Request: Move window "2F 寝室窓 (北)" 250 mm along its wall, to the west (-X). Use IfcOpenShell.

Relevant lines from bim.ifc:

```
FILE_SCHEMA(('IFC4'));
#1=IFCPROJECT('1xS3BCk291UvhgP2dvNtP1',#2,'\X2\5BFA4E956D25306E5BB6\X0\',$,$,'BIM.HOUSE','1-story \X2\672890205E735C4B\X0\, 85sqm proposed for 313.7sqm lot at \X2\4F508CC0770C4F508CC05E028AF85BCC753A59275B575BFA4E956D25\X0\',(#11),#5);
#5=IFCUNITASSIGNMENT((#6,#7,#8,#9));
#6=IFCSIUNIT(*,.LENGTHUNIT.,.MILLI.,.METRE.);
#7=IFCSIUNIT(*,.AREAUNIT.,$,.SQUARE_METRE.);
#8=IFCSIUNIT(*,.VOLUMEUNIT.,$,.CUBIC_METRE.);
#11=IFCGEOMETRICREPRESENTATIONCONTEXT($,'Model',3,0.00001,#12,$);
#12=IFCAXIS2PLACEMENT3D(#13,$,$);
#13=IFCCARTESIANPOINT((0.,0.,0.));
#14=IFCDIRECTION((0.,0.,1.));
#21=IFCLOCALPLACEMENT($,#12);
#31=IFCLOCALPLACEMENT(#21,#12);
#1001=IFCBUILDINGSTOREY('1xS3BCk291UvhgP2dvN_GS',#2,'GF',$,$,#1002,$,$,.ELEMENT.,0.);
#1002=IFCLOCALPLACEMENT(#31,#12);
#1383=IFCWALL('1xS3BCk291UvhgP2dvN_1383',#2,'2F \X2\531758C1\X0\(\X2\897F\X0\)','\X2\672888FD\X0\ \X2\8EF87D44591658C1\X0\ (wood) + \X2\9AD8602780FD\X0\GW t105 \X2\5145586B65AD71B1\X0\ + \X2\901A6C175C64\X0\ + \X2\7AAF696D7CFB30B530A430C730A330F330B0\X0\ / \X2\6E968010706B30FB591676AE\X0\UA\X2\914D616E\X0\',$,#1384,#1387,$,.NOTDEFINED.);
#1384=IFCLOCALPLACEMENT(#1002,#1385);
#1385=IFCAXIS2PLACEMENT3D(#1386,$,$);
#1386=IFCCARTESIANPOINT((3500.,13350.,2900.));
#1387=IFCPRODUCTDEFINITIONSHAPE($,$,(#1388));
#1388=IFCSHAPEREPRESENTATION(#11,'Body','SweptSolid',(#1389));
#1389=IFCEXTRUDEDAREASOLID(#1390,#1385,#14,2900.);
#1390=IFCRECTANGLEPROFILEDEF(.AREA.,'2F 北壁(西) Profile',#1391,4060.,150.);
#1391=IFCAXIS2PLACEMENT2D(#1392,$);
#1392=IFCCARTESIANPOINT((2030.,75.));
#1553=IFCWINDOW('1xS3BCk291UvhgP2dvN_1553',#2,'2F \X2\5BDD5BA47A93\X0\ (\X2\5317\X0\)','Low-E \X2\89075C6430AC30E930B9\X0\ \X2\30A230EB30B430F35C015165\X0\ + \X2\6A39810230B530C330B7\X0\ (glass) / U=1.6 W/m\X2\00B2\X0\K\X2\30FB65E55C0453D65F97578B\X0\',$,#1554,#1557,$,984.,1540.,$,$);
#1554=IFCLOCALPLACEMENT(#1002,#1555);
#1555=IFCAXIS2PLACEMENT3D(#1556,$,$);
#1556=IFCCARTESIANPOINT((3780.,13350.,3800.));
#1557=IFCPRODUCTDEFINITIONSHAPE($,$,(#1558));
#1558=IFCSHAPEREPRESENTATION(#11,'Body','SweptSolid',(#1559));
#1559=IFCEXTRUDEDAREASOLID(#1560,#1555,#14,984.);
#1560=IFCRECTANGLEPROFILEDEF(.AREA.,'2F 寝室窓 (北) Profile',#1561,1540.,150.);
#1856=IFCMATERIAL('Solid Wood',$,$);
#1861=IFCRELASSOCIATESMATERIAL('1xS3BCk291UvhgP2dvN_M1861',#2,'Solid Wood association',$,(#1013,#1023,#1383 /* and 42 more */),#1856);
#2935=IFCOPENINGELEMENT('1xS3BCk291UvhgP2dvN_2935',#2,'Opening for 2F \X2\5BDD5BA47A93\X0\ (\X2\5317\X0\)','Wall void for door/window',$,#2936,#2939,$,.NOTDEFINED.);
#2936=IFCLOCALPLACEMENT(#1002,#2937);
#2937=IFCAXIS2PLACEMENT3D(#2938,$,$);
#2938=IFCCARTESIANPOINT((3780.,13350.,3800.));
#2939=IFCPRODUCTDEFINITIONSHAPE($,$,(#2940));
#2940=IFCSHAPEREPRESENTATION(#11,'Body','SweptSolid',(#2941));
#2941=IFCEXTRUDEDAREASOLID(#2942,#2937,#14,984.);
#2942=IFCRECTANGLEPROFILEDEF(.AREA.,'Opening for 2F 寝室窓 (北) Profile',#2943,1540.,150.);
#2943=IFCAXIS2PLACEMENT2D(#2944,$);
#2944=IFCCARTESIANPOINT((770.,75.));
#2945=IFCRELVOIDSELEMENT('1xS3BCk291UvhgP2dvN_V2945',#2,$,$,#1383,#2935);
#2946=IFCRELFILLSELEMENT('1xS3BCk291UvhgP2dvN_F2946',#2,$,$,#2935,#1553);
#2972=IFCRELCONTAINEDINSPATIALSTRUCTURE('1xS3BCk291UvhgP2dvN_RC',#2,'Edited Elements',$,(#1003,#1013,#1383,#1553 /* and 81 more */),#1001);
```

```python
import ifcopenshell
import ifcopenshell.api.geometry
import ifcopenshell.util.placement
import ifcopenshell.util.unit

model = ifcopenshell.open("bim.ifc")
unit_scale = ifcopenshell.util.unit.calculate_unit_scale(model)

window = model.by_guid("1xS3BCk291UvhgP2dvN_1553")
opening = window.FillsVoids[0].RelatingOpeningElement
wall = opening.VoidsElements[0].RelatingBuildingElement

wall_matrix = ifcopenshell.util.placement.get_local_placement(wall.ObjectPlacement)
shift = wall_matrix[:3, 0] * -0.25 / unit_scale
before = ifcopenshell.util.placement.get_local_placement(window.ObjectPlacement)[:3, 3].copy()

# The window is not placed relative to its opening, so move both.
for product in (opening, window):
    matrix = ifcopenshell.util.placement.get_local_placement(product.ObjectPlacement)
    matrix[:3, 3] += shift
    ifcopenshell.api.geometry.edit_object_placement(model, product=product, matrix=matrix, is_si=False)

after = ifcopenshell.util.placement.get_local_placement(window.ObjectPlacement)[:3, 3]
print("window moved by", (after - before).round(3) + 0.0)

model.write("bim_updated.ifc")
```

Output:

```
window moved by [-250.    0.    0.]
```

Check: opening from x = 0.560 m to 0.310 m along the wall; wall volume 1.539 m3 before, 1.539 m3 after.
